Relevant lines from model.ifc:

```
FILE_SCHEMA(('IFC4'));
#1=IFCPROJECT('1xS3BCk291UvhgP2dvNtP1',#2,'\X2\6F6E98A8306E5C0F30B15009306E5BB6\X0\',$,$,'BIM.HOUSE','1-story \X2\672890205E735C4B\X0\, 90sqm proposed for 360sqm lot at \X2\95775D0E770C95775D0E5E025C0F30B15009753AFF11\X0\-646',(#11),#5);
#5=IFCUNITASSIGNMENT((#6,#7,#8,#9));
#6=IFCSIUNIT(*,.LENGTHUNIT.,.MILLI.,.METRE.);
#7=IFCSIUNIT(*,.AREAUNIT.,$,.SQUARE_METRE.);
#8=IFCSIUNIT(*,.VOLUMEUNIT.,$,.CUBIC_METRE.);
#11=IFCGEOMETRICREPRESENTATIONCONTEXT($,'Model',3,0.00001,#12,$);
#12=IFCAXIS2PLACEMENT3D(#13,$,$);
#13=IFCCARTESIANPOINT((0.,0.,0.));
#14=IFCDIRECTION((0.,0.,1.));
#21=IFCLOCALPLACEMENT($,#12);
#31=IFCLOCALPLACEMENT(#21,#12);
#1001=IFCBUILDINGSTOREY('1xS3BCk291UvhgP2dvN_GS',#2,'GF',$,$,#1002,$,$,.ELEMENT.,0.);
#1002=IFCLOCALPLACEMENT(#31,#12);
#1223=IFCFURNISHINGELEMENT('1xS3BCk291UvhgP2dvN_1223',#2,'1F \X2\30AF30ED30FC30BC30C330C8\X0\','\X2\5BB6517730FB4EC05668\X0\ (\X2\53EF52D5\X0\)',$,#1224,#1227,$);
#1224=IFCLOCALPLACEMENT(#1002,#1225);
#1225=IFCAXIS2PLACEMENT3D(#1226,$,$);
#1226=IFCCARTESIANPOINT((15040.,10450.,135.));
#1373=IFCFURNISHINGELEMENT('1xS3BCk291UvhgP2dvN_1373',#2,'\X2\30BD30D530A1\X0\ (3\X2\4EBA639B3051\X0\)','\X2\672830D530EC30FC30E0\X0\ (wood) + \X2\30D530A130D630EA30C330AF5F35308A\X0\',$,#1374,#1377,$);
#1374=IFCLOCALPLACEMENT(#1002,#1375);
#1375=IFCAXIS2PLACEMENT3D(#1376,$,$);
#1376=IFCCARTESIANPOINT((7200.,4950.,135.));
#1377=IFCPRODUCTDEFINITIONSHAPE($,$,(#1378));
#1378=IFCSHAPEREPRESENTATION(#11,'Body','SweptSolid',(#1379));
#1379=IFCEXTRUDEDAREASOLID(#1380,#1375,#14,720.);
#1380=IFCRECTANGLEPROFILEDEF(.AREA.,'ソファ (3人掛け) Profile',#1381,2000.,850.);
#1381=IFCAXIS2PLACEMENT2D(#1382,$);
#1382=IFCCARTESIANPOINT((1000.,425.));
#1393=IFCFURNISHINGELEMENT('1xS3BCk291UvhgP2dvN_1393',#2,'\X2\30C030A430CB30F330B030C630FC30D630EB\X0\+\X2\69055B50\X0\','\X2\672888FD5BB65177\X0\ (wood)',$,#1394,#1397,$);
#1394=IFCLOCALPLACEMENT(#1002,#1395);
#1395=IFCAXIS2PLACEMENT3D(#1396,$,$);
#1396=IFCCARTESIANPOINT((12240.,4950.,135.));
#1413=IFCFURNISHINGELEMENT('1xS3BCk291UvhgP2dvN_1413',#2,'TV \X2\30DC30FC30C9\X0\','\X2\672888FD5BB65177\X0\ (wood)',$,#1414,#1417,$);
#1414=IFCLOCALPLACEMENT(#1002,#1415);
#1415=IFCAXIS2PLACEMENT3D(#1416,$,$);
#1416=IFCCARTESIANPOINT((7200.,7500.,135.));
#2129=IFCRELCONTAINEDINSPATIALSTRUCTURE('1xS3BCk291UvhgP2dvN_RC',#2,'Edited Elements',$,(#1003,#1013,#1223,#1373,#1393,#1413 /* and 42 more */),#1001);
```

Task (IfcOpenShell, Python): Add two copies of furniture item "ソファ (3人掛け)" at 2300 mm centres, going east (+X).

```python
import numpy as np
import ifcopenshell
import ifcopenshell.api.geometry
import ifcopenshell.api.root
import ifcopenshell.util.element
import ifcopenshell.util.placement
import ifcopenshell.util.unit

model = ifcopenshell.open("model.ifc")
unit_scale = ifcopenshell.util.unit.calculate_unit_scale(model)


def reuse_history(source, copy):
    """copy_class also copies each property set's owner history, people and application; keep the originals."""
    for rel in copy.IsDefinedBy:
        if rel.is_a("IfcRelDefinesByProperties") and (history := rel.RelatingPropertyDefinition.OwnerHistory):
            rel.RelatingPropertyDefinition.OwnerHistory = source.OwnerHistory
            ifcopenshell.util.element.remove_deep2(model, history)


source = model.by_guid("1xS3BCk291UvhgP2dvN_1373")
base = ifcopenshell.util.placement.get_local_placement(source.ObjectPlacement)
step = np.array([1.0, 0.0, 0.0]) * 2.3 / unit_scale

for i in range(1, 3):
    copy = ifcopenshell.api.root.copy_class(model, product=source)
    copy.Representation = ifcopenshell.util.element.copy_deep(
        model, source.Representation, exclude=["IfcGeometricRepresentationContext", "IfcRepresentationMap"]
    )
    reuse_history(source, copy)
    matrix = base.copy()
    matrix[:3, 3] += i * step
    print("added at", matrix[:3, 3].round(3) + 0.0)
    ifcopenshell.api.geometry.edit_object_placement(model, product=copy, matrix=matrix, is_si=False)

model.write("model_edited.ifc")
```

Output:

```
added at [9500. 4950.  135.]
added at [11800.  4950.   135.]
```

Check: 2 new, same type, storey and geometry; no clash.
